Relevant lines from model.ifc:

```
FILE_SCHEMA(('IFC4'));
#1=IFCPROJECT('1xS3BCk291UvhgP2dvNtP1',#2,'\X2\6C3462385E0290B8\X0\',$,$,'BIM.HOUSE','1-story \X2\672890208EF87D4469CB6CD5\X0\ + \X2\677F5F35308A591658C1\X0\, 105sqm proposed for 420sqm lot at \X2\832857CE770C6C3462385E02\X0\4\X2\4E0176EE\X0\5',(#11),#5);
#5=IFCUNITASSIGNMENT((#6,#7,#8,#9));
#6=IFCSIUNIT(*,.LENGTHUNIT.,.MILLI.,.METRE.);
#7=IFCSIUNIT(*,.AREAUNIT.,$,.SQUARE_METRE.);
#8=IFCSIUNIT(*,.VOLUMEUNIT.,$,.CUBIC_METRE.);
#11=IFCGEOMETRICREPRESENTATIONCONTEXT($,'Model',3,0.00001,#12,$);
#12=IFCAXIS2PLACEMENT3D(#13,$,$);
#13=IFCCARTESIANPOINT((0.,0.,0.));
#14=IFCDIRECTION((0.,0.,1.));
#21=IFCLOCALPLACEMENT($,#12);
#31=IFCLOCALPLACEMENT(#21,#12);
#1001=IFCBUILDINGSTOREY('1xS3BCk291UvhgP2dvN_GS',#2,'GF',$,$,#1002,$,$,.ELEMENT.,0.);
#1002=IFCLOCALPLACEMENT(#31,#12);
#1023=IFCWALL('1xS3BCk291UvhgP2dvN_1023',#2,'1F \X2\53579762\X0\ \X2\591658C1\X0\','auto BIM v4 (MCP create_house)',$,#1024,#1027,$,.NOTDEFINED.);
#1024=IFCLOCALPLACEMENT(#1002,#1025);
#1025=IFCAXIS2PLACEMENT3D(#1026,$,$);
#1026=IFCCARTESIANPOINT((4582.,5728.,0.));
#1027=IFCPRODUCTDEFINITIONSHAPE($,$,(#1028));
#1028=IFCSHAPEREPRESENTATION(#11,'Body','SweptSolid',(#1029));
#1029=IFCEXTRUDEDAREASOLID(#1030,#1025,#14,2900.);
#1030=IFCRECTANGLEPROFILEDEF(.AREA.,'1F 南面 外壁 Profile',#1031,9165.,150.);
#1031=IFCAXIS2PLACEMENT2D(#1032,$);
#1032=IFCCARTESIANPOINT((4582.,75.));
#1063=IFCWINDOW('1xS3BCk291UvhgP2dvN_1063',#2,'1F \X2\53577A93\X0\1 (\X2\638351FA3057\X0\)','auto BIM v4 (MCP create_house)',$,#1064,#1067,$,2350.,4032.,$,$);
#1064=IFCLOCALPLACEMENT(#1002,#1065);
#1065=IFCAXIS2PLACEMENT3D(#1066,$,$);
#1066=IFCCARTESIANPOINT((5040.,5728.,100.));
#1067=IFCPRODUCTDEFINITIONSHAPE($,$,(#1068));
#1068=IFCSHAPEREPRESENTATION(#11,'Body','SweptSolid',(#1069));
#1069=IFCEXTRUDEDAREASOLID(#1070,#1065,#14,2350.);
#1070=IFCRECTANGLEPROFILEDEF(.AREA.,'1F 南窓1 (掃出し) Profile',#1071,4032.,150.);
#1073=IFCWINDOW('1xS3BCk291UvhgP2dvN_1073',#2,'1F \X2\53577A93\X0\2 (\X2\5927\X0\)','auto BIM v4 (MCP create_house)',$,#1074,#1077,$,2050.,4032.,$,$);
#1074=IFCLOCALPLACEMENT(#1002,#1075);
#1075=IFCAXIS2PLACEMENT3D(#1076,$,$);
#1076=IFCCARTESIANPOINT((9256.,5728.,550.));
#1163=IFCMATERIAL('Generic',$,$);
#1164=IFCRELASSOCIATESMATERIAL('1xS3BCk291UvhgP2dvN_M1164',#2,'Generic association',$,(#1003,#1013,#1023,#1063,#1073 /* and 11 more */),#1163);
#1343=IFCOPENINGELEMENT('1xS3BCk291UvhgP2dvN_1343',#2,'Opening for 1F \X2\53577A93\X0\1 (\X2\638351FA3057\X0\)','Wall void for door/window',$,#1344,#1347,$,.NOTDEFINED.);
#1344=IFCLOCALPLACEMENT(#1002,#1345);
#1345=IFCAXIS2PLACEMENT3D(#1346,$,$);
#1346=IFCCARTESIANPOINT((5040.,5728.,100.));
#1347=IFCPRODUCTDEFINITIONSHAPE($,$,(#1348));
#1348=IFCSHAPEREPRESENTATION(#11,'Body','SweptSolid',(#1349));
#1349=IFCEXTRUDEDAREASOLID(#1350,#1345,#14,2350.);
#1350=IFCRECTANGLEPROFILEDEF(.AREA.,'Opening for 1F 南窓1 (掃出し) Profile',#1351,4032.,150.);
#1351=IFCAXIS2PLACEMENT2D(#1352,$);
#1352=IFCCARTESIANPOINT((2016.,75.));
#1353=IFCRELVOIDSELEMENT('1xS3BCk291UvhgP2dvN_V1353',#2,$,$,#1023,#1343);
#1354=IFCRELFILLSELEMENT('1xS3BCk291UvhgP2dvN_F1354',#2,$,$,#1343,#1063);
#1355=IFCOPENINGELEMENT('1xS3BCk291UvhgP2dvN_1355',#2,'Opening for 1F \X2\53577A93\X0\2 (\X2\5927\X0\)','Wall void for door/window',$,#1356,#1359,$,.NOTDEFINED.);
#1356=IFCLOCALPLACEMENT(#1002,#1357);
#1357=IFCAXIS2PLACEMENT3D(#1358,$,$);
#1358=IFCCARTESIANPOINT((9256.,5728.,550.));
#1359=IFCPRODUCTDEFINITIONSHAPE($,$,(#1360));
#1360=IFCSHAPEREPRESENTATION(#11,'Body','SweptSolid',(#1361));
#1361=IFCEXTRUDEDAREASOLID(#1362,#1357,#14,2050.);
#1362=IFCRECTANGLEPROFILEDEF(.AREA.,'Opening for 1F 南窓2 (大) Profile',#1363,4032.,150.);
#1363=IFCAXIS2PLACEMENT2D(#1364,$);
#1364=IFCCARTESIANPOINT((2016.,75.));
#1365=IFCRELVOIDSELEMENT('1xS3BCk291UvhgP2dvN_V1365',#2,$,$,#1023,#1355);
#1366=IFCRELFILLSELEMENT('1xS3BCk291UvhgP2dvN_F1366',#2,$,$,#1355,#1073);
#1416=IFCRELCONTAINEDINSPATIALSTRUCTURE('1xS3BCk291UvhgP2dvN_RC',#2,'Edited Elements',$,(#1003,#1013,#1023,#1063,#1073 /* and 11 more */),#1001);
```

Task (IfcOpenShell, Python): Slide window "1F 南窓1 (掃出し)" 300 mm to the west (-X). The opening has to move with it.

```python
import ifcopenshell
import ifcopenshell.api.geometry
import ifcopenshell.util.placement

model = ifcopenshell.open("model.ifc")

window = model.by_guid("1xS3BCk291UvhgP2dvN_1063")
opening = window.FillsVoids[0].RelatingOpeningElement
wall = opening.VoidsElements[0].RelatingBuildingElement

wall_matrix = ifcopenshell.util.placement.get_local_placement(wall.ObjectPlacement)
shift = wall_matrix[:3, 0] * -300.0
before = ifcopenshell.util.placement.get_local_placement(window.ObjectPlacement)[:3, 3].copy()

# The window is not placed relative to its opening, so move both.
for product in (opening, window):
    matrix = ifcopenshell.util.placement.get_local_placement(product.ObjectPlacement)
    matrix[:3, 3] += shift
    ifcopenshell.api.geometry.edit_object_placement(model, product=product, matrix=matrix, is_si=False)

after = ifcopenshell.util.placement.get_local_placement(window.ObjectPlacement)[:3, 3]
print("window moved by", (after - before).round(3) + 0.0)

model.write("model_edited.ifc")
```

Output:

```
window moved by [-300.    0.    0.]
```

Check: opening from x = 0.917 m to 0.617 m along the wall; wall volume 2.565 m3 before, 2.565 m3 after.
